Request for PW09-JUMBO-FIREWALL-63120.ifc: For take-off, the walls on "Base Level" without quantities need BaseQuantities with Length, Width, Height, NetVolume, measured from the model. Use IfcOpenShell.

First a look at what the model holds.

```python
import ifcopenshell
import ifcopenshell.util.element
import ifcopenshell.util.unit

model = ifcopenshell.open("PW09-JUMBO-FIREWALL-63120.ifc")
print(model.schema)
for unit_type in ("LENGTHUNIT", "AREAUNIT", "VOLUMEUNIT"):
    print(unit_type, ifcopenshell.util.unit.calculate_unit_scale(model, unit_type))
storey = next(s for s in model.by_type("IfcBuildingStorey") if s.Name == "Base Level")
walls = [e for e in ifcopenshell.util.element.get_decomposition(storey) if e.is_a("IfcWall")]
for e in sorted(walls, key=lambda e: e.id()):
    print(e.id(), e.is_a(), e.Name, list(ifcopenshell.util.element.get_psets(e, qtos_only=True)), sep=" | ")
```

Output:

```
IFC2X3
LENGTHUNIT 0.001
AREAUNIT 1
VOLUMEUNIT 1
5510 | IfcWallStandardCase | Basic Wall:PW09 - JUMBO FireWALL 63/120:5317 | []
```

```python
import ifcopenshell
import ifcopenshell.api.pset
import ifcopenshell.geom
import ifcopenshell.util.element
import ifcopenshell.util.shape
import ifcopenshell.util.unit

model = ifcopenshell.open("PW09-JUMBO-FIREWALL-63120.ifc")
unit_scale = ifcopenshell.util.unit.calculate_unit_scale(model)
volume_scale = ifcopenshell.util.unit.calculate_unit_scale(model, "VOLUMEUNIT")
settings = ifcopenshell.geom.settings()

storey = next(s for s in model.by_type("IfcBuildingStorey") if s.Name == "Base Level")
walls = [e for e in ifcopenshell.util.element.get_decomposition(storey) if e.is_a("IfcWall")]

for e in sorted(walls, key=lambda e: e.id()):
    if ifcopenshell.util.element.get_psets(e, qtos_only=True, should_inherit=False):
        continue
    # Geometry comes back in metres, in the element's own axes.
    shape = ifcopenshell.geom.create_shape(settings, e)
    values = {
        "Length": ifcopenshell.util.shape.get_x(shape.geometry) / unit_scale,
        "Width": ifcopenshell.util.shape.get_y(shape.geometry) / unit_scale,
        "Height": ifcopenshell.util.shape.get_z(shape.geometry) / unit_scale,
        "NetVolume": ifcopenshell.util.shape.get_volume(shape.geometry) / volume_scale,
    }
    qto = ifcopenshell.api.pset.add_qto(model, product=e, name="BaseQuantities")
    ifcopenshell.api.pset.edit_qto(model, qto=qto, properties=values)
    print(e.id(), {k: round(v, 3) for k, v in values.items()})

model.write("PW09-JUMBO-FIREWALL-63120_v2.ifc")
```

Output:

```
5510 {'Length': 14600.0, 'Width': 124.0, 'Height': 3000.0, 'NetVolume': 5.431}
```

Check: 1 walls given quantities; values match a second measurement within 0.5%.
